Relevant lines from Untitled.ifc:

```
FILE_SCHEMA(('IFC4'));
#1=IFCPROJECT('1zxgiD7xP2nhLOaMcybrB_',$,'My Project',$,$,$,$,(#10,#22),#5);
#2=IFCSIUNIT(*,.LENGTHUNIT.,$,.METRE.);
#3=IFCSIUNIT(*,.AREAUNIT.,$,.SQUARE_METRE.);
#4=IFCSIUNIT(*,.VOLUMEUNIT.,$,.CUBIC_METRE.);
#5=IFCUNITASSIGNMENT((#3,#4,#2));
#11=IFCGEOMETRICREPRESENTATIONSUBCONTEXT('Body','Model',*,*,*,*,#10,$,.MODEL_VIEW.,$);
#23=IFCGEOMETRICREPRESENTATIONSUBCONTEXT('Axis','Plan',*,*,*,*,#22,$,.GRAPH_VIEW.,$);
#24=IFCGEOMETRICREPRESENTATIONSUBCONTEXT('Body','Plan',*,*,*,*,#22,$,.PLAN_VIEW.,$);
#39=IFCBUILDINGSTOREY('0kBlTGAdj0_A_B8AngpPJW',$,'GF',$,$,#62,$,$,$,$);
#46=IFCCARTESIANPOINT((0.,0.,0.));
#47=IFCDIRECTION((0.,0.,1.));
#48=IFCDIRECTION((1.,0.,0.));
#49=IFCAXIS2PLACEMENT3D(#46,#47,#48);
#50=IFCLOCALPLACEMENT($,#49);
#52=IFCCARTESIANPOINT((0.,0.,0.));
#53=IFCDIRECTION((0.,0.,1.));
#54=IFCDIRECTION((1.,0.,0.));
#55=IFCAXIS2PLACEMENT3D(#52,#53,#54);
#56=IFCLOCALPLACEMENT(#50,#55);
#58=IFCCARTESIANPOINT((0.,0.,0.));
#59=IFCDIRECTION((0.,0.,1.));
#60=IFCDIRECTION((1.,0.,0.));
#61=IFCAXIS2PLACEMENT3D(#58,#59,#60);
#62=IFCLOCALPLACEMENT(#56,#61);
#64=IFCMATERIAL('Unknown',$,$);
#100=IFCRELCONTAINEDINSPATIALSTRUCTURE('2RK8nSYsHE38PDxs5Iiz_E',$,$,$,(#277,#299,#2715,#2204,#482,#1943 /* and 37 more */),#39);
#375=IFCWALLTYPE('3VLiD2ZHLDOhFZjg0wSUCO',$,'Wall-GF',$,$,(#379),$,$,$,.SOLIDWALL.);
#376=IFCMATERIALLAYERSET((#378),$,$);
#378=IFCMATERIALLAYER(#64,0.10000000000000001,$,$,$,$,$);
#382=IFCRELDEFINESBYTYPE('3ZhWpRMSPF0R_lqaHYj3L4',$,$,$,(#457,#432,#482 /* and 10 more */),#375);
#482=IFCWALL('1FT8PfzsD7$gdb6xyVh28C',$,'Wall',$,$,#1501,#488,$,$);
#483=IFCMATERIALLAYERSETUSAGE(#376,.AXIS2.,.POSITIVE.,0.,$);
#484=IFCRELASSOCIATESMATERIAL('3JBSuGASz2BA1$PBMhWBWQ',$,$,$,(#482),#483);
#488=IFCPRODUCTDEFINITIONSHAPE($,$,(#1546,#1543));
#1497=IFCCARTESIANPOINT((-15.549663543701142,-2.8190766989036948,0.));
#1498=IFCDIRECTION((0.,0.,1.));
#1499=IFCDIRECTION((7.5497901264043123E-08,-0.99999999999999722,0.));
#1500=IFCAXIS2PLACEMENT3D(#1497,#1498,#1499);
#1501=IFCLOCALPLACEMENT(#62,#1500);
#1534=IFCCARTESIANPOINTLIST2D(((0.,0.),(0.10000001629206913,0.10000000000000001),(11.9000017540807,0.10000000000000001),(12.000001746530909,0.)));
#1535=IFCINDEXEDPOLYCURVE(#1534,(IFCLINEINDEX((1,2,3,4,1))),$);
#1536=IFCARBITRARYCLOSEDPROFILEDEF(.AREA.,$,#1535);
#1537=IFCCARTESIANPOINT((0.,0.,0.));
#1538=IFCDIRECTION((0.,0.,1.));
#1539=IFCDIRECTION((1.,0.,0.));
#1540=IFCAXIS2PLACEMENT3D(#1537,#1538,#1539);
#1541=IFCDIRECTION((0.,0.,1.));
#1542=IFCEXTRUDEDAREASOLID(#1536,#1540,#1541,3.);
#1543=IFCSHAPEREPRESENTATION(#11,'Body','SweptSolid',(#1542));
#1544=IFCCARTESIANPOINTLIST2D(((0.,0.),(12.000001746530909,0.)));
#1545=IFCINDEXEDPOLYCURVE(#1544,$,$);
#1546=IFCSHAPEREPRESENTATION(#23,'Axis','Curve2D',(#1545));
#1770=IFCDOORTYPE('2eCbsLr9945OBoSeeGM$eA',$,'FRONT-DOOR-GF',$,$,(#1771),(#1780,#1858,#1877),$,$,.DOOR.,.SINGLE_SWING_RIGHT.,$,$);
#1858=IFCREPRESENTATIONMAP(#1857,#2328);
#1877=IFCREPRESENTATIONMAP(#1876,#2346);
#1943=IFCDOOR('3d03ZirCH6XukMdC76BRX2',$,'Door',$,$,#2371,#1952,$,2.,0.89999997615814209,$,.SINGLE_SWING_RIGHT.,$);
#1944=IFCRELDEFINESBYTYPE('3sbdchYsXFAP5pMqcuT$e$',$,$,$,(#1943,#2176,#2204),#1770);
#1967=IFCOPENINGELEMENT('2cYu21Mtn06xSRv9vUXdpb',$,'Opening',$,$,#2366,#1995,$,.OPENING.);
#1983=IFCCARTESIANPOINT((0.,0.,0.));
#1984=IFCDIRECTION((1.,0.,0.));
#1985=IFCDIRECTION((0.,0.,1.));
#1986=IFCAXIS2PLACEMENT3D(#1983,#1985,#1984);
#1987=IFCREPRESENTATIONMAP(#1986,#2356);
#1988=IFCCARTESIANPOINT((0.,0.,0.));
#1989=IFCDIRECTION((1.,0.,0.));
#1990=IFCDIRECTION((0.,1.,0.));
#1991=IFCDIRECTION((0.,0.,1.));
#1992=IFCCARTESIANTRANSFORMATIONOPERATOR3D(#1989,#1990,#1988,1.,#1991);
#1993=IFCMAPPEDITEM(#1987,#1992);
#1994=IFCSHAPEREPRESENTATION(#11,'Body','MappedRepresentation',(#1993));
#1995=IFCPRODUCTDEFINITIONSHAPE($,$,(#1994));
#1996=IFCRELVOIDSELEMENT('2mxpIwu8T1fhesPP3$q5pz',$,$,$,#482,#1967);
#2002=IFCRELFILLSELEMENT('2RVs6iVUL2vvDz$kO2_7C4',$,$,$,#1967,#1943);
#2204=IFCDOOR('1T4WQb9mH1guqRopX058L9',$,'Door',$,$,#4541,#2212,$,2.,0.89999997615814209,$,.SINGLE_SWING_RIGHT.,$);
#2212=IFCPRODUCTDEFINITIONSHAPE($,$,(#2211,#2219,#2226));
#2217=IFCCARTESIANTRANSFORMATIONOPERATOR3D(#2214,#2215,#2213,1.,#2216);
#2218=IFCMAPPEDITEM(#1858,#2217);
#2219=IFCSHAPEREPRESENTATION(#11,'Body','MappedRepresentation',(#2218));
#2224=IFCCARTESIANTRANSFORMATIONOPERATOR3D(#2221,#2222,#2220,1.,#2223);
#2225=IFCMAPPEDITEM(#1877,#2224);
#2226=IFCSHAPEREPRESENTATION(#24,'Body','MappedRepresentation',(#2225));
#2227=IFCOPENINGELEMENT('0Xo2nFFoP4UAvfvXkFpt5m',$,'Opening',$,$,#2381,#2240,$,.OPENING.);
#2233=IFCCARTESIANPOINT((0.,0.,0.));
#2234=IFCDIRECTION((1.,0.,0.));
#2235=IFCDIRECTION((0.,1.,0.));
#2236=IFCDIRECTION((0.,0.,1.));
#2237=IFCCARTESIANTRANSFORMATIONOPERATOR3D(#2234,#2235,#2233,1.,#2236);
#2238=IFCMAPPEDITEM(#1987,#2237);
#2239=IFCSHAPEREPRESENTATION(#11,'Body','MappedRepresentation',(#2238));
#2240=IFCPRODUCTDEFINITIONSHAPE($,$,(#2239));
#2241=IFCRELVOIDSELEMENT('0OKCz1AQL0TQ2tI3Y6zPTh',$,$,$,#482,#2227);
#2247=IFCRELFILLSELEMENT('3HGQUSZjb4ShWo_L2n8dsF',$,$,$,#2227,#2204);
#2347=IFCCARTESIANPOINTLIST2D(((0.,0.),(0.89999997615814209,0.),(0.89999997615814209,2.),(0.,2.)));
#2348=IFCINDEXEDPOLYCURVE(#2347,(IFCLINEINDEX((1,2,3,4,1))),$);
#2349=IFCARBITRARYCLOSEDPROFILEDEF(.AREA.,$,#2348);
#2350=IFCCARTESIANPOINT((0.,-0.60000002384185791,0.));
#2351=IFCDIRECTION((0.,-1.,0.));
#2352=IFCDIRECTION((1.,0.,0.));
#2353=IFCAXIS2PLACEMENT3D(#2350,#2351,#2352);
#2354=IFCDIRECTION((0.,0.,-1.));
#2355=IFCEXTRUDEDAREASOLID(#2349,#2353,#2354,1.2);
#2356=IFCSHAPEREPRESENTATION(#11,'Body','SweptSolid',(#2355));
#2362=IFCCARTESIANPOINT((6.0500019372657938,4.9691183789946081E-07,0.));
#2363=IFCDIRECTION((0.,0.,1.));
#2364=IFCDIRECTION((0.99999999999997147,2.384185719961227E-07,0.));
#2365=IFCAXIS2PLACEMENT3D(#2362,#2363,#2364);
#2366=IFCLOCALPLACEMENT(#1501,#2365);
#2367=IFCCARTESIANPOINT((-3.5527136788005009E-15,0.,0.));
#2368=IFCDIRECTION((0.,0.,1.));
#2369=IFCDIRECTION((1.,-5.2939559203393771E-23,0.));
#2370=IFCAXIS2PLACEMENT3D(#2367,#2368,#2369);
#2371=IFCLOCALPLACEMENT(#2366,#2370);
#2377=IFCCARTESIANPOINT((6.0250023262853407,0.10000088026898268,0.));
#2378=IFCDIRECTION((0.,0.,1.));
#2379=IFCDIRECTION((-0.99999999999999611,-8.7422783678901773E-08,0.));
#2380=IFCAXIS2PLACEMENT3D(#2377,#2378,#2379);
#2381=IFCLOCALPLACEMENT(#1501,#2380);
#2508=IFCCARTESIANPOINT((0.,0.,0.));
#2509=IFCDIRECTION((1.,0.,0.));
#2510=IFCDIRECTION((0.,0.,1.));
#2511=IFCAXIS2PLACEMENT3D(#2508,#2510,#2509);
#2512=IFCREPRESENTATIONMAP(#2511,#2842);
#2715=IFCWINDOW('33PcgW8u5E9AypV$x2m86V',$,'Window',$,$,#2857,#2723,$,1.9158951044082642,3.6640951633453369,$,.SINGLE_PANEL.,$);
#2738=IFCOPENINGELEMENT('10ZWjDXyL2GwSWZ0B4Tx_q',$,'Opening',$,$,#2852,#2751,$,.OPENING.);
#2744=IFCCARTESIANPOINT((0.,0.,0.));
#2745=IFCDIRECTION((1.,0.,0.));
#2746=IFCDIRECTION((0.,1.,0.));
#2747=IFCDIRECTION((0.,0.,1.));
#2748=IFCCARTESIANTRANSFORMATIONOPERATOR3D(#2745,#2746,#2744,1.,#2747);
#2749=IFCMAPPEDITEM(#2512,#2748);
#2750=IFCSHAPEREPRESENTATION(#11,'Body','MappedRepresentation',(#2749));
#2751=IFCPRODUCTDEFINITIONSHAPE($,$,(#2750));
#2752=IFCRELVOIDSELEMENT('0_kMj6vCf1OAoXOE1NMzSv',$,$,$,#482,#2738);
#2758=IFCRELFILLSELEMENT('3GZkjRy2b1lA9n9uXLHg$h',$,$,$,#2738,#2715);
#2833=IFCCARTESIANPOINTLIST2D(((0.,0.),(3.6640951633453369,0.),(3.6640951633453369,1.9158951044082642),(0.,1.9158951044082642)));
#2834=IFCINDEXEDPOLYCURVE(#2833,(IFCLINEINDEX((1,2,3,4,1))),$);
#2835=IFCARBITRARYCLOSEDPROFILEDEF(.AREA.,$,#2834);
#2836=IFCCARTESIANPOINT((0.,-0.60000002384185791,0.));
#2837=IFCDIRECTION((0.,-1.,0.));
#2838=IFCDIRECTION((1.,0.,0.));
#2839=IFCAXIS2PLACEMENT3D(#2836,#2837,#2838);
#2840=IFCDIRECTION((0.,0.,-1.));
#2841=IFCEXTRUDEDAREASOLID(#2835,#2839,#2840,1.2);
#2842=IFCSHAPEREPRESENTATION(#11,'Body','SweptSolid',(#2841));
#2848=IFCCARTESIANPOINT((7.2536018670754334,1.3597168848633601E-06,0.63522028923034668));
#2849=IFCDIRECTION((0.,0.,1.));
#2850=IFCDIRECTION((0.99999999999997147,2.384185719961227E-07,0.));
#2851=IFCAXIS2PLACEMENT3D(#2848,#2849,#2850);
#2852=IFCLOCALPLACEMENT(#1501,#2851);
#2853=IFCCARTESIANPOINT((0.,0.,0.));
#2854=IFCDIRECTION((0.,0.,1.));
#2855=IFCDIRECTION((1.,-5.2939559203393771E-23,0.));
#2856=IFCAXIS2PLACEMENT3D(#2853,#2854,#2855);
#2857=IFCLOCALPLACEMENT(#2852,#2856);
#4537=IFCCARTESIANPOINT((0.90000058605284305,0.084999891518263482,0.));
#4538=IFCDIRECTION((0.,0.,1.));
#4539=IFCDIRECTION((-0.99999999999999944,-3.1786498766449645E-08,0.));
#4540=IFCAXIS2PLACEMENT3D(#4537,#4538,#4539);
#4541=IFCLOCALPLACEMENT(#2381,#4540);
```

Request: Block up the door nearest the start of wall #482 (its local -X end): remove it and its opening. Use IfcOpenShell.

```python
import ifcopenshell
import ifcopenshell.api.feature
import ifcopenshell.api.root
import ifcopenshell.geom
import ifcopenshell.util.shape

model = ifcopenshell.open("Untitled.ifc")
settings = ifcopenshell.geom.settings()


def volume(element):
    """Net volume in cubic metres, openings subtracted."""
    shape = ifcopenshell.geom.create_shape(settings, element)
    return ifcopenshell.util.shape.get_volume(shape.geometry)


door = model.by_guid("1T4WQb9mH1guqRopX058L9")
opening = door.FillsVoids[0].RelatingOpeningElement
wall = opening.VoidsElements[0].RelatingBuildingElement
before = volume(wall)

ifcopenshell.api.root.remove_product(model, product=door)
ifcopenshell.api.feature.remove_feature(model, feature=opening)

after = volume(wall)

print(f"wall volume {before:.3f} -> {after:.3f} m3")

model.write("Untitled_updated.ifc")
```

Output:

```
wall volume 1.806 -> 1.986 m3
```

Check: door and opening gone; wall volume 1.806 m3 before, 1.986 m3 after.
